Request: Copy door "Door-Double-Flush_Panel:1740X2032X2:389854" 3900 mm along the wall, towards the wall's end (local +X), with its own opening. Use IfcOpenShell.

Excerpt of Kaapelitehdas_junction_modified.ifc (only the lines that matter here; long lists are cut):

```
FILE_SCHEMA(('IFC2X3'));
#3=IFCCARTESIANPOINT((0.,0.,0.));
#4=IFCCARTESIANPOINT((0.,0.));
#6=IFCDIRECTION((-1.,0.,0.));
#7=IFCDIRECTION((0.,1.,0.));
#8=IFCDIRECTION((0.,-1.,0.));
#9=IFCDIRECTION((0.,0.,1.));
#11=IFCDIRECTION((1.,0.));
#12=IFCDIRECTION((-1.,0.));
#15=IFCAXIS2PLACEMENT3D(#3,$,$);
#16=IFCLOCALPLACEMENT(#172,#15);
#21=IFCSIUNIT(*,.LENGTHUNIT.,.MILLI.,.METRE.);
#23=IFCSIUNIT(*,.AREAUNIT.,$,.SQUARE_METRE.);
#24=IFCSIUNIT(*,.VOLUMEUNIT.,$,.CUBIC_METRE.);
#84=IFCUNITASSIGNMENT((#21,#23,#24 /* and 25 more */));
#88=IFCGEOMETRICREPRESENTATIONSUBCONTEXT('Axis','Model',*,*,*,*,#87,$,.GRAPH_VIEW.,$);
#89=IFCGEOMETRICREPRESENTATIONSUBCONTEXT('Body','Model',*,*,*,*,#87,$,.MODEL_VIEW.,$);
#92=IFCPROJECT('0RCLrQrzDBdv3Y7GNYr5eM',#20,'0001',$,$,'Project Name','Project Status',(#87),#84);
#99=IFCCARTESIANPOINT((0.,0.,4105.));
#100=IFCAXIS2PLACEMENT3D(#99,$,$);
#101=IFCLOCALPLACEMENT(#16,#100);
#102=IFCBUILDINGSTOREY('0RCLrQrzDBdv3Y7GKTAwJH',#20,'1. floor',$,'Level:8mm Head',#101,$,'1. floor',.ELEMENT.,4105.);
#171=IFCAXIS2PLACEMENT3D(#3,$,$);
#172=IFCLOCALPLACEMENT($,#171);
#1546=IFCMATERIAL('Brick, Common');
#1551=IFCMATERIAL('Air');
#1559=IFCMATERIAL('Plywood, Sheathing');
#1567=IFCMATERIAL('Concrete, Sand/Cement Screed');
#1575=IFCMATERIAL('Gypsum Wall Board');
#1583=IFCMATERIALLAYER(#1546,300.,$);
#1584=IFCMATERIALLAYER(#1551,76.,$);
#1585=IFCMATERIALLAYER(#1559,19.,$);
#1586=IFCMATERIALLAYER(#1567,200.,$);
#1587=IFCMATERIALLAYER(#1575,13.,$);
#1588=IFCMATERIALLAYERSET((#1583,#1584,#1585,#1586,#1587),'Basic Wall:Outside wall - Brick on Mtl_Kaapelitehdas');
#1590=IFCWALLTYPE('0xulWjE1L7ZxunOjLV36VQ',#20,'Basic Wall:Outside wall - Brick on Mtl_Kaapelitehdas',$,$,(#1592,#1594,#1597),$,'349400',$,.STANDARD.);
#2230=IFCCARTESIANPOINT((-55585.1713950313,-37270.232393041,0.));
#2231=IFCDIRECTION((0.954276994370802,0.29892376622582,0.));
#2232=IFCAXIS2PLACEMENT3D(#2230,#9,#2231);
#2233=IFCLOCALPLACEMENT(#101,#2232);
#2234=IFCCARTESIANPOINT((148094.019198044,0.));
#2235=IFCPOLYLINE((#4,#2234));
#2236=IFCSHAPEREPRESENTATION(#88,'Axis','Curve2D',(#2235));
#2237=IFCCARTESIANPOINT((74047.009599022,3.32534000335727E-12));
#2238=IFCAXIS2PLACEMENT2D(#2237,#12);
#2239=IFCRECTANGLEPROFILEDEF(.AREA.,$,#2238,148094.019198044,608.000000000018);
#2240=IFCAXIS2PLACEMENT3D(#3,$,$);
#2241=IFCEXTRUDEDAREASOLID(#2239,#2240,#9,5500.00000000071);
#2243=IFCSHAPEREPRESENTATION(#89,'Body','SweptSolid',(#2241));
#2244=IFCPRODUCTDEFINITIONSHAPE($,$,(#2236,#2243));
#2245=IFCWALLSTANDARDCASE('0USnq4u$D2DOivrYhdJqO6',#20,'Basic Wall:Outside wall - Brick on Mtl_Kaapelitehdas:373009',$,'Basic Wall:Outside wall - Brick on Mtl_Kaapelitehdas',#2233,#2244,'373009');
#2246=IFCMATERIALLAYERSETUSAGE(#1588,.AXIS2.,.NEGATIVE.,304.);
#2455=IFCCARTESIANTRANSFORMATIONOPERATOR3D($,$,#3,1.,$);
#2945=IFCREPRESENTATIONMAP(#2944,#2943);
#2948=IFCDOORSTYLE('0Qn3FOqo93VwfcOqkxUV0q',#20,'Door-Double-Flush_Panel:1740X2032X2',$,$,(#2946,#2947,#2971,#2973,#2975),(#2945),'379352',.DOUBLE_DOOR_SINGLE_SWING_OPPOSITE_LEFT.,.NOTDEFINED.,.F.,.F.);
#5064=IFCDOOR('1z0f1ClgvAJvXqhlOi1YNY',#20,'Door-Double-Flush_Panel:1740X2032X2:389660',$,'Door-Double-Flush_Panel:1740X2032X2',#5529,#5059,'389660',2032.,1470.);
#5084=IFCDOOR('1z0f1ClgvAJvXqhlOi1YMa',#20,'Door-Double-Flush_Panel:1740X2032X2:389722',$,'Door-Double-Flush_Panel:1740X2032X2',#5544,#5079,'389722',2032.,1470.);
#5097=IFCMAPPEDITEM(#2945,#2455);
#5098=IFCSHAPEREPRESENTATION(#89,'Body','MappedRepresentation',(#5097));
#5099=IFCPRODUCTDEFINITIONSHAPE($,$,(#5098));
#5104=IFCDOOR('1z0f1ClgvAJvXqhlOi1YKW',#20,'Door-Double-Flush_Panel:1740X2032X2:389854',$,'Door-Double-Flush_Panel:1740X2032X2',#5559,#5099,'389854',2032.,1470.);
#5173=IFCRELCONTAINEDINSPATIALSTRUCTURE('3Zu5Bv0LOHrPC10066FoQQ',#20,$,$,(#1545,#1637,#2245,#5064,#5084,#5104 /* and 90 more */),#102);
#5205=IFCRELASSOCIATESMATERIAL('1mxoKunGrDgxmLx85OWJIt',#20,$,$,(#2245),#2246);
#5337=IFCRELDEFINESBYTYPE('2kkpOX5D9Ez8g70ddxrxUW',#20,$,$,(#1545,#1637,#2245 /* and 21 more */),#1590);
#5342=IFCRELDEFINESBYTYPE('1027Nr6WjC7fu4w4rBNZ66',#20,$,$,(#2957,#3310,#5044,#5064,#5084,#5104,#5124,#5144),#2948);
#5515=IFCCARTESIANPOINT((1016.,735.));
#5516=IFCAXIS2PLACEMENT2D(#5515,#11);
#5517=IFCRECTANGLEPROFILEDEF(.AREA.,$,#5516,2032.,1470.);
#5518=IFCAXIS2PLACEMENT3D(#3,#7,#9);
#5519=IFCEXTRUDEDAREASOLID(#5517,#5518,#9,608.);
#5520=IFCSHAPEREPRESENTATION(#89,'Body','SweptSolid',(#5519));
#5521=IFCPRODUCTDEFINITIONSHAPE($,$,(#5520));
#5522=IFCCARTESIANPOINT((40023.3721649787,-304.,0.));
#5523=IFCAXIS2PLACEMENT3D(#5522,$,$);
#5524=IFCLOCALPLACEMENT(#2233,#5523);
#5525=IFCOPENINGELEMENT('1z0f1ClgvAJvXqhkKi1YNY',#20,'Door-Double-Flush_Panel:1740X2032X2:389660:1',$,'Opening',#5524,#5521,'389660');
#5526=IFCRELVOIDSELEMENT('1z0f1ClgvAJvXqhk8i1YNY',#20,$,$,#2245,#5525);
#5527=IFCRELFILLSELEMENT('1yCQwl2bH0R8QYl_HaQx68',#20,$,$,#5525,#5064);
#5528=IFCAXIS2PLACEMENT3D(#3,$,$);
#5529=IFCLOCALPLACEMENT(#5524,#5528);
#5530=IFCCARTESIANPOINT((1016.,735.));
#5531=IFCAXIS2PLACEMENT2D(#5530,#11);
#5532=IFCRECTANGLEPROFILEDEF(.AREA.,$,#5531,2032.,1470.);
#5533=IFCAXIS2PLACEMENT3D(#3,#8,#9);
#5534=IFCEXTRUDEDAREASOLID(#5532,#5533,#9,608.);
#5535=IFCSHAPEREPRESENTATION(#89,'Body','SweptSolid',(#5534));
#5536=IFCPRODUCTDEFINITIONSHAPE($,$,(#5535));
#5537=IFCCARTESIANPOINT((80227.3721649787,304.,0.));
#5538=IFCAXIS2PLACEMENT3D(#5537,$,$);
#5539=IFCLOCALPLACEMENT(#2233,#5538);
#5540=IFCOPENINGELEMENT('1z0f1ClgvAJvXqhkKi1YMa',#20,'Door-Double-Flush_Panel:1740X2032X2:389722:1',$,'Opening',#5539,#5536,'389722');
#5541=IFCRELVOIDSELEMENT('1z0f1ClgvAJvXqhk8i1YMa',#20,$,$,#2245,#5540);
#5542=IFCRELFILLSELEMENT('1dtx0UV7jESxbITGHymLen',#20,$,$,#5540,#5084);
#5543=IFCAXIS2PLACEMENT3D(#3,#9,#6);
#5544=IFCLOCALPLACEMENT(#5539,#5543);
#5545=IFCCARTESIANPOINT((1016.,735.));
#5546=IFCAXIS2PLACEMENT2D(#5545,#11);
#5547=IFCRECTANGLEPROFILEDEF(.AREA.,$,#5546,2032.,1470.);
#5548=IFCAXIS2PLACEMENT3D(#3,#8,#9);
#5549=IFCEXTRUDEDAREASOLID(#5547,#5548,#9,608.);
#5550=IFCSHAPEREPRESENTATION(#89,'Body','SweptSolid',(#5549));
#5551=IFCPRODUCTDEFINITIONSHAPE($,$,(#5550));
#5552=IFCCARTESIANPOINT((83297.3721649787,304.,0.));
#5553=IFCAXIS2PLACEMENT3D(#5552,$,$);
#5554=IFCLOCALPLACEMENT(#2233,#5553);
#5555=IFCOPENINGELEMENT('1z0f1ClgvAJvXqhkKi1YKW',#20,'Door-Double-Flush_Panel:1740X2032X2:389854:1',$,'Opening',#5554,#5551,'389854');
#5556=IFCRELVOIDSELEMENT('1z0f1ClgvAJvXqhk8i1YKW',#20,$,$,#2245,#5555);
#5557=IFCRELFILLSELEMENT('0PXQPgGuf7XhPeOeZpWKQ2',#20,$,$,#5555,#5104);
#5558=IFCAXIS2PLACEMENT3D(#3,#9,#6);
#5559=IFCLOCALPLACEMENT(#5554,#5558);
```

```python
import ifcopenshell
import ifcopenshell.api.feature
import ifcopenshell.api.geometry
import ifcopenshell.api.root
import ifcopenshell.geom
import ifcopenshell.util.element
import ifcopenshell.util.placement
import ifcopenshell.util.shape
import ifcopenshell.util.unit

model = ifcopenshell.open("Kaapelitehdas_junction_modified.ifc")
unit_scale = ifcopenshell.util.unit.calculate_unit_scale(model)
settings = ifcopenshell.geom.settings()


def volume(element):
    """Net volume in cubic metres, openings subtracted."""
    shape = ifcopenshell.geom.create_shape(settings, element)
    return ifcopenshell.util.shape.get_volume(shape.geometry)


def reuse_history(source, copy):
    """copy_class also copies each property set's owner history, people and application; keep the originals."""
    for rel in copy.IsDefinedBy:
        if rel.is_a("IfcRelDefinesByProperties") and (history := rel.RelatingPropertyDefinition.OwnerHistory):
            rel.RelatingPropertyDefinition.OwnerHistory = source.OwnerHistory
            ifcopenshell.util.element.remove_deep2(model, history)


door = model.by_guid("1z0f1ClgvAJvXqhlOi1YKW")
opening = door.FillsVoids[0].RelatingOpeningElement
wall = opening.VoidsElements[0].RelatingBuildingElement
before = volume(wall)
shift = ifcopenshell.util.placement.get_local_placement(wall.ObjectPlacement)[:3, 0] * 3.9 / unit_scale

# copy_class copies the void relationship, type, container and properties, but no geometry.
new_opening = ifcopenshell.api.root.copy_class(model, product=opening)
new_opening.Representation = ifcopenshell.util.element.copy_deep(
    model, opening.Representation, exclude=["IfcGeometricRepresentationContext", "IfcRepresentationMap"]
)
new_opening.Name = "Door-Double-Flush_Panel:1740X2032X2"
new_opening.Tag = None
new_door = ifcopenshell.api.root.copy_class(model, product=door)
new_door.Representation = ifcopenshell.util.element.copy_deep(
    model, door.Representation, exclude=["IfcGeometricRepresentationContext", "IfcRepresentationMap"]
)
new_door.Name = "Door-Double-Flush_Panel:1740X2032X2"
new_door.Tag = None
reuse_history(door, new_door)
fills = ifcopenshell.api.feature.add_filling(model, opening=new_opening, element=new_door)
fills.OwnerHistory = new_door.OwnerHistory  # required in IFC2X3

for old, new in ((opening, new_opening), (door, new_door)):
    matrix = ifcopenshell.util.placement.get_local_placement(old.ObjectPlacement)
    matrix[:3, 3] += shift
    ifcopenshell.api.geometry.edit_object_placement(model, product=new, matrix=matrix, is_si=False)

after = volume(wall)

print(f"wall volume {before:.3f} -> {after:.3f} m3")

model.write("Kaapelitehdas_junction_modified_rev.ifc")
```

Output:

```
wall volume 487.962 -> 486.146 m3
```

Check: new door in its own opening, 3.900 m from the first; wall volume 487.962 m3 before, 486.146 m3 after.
